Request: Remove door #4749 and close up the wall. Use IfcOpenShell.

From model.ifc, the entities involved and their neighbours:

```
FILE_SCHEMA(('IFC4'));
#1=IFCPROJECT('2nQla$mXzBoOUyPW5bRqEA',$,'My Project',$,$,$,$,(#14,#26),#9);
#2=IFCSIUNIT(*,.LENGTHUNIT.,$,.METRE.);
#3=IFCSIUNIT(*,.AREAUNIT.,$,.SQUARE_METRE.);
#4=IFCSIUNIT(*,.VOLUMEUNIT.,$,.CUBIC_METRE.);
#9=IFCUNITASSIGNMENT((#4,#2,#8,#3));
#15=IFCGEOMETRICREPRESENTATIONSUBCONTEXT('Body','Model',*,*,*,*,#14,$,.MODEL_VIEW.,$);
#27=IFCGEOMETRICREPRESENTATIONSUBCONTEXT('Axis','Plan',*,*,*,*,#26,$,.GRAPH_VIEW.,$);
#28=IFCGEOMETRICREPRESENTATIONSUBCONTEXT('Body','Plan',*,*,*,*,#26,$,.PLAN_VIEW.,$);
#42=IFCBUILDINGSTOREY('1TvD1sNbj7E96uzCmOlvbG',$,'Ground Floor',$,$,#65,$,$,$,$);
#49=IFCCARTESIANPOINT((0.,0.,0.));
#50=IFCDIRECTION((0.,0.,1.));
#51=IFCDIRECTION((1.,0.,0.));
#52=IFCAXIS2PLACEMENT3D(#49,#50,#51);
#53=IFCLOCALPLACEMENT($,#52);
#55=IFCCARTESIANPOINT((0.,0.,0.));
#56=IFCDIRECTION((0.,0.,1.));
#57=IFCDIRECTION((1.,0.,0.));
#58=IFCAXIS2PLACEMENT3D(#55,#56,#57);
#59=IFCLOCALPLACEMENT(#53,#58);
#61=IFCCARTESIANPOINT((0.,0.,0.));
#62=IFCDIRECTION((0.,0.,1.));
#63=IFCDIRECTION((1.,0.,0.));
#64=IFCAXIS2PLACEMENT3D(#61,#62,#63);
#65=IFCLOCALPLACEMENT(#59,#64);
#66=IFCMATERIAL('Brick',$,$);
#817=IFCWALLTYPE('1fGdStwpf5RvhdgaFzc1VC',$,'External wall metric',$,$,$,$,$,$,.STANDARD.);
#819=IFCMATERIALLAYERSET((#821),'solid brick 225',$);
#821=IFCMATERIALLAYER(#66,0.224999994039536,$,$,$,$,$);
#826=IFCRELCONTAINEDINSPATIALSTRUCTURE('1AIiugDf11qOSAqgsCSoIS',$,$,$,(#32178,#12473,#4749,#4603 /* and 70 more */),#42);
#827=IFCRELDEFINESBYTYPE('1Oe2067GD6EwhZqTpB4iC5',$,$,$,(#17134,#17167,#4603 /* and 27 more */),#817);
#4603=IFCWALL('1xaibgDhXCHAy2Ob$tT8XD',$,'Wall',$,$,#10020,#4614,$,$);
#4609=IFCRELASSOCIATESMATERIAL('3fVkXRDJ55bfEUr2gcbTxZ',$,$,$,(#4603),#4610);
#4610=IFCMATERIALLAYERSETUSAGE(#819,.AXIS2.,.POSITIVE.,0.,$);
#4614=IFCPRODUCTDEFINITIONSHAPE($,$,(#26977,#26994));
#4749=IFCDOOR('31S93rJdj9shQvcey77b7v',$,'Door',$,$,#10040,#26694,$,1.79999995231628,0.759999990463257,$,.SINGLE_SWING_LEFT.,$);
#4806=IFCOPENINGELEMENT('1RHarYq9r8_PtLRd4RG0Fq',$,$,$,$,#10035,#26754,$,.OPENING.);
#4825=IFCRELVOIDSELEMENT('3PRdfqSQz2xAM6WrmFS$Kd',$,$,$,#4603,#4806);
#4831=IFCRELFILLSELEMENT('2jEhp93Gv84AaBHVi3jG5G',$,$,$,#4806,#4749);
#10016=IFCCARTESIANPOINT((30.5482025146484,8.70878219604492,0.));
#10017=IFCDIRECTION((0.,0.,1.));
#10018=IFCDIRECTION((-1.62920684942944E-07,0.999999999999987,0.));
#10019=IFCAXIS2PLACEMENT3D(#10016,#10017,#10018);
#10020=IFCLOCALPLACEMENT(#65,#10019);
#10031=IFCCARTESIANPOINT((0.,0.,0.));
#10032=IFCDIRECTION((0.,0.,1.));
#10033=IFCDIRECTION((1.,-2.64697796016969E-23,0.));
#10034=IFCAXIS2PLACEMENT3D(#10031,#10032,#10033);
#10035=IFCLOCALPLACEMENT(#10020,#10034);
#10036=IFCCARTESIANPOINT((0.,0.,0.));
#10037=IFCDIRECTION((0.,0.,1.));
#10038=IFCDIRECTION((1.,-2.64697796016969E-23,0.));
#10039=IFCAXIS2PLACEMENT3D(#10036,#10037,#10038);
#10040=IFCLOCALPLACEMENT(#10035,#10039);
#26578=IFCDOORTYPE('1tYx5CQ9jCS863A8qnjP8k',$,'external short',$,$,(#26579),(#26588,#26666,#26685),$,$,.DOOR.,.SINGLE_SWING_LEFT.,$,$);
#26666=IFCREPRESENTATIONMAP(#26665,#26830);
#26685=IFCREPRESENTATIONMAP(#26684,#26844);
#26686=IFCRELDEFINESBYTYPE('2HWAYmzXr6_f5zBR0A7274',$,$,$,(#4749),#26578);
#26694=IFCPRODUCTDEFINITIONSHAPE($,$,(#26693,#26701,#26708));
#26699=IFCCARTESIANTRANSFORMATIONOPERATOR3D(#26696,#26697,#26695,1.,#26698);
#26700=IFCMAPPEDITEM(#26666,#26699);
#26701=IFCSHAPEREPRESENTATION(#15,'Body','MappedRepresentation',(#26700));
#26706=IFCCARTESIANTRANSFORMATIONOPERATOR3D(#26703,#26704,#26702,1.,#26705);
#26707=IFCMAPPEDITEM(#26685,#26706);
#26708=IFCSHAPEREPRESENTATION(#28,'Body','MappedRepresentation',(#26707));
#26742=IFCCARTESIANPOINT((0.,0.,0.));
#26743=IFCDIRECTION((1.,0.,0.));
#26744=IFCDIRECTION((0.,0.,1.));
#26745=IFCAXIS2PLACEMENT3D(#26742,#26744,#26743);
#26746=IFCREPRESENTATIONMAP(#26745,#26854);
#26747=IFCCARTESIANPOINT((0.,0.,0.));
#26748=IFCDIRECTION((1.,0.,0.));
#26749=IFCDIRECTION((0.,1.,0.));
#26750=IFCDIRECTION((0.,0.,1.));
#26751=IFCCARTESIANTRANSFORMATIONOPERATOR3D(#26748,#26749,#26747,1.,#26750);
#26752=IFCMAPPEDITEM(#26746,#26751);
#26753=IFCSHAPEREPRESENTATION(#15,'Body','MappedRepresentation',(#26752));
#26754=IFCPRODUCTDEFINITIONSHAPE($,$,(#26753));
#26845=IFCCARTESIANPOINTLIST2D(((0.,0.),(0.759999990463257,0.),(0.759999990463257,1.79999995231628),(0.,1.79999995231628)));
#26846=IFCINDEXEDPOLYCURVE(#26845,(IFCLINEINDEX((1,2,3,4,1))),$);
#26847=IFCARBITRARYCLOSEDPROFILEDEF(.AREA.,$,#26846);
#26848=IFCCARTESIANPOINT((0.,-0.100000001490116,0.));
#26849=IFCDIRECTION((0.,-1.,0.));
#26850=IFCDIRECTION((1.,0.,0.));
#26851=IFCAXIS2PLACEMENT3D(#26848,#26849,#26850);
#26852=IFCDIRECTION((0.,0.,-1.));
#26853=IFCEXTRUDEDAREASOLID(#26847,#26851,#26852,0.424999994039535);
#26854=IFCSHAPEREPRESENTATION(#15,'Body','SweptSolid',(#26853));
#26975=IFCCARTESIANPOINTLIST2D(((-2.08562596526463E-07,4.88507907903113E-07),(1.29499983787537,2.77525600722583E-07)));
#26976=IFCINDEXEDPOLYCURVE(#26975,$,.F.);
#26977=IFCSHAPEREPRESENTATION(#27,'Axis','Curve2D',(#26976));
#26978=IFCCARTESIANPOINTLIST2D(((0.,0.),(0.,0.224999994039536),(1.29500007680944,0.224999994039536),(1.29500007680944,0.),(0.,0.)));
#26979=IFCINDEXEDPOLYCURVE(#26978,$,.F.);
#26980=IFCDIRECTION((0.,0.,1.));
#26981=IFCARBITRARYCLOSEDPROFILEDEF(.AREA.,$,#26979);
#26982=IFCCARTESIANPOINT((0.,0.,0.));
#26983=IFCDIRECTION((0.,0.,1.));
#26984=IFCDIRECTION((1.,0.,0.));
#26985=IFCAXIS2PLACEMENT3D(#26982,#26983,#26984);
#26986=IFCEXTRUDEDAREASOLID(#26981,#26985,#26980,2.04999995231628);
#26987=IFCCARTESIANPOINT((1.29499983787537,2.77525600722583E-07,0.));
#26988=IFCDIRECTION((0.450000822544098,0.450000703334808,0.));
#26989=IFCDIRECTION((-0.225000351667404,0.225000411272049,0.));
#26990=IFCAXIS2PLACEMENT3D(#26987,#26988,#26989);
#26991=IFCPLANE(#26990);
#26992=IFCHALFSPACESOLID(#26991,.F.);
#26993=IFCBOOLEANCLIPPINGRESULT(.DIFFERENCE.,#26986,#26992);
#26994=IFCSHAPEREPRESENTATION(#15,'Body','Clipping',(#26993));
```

```python
import ifcopenshell
import ifcopenshell.api.feature
import ifcopenshell.api.root
import ifcopenshell.geom
import ifcopenshell.util.shape

model = ifcopenshell.open("model.ifc")
settings = ifcopenshell.geom.settings()


def volume(element):
    """Net volume in cubic metres, openings subtracted."""
    shape = ifcopenshell.geom.create_shape(settings, element)
    return ifcopenshell.util.shape.get_volume(shape.geometry)


door = model.by_guid("31S93rJdj9shQvcey77b7v")
opening = door.FillsVoids[0].RelatingOpeningElement
wall = opening.VoidsElements[0].RelatingBuildingElement
before = volume(wall)

ifcopenshell.api.root.remove_product(model, product=door)
ifcopenshell.api.feature.remove_feature(model, feature=opening)

after = volume(wall)

print(f"wall volume {before:.3f} -> {after:.3f} m3")

model.write("model-out.ifc")
```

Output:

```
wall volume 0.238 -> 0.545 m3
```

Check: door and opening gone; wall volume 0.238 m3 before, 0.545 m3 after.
